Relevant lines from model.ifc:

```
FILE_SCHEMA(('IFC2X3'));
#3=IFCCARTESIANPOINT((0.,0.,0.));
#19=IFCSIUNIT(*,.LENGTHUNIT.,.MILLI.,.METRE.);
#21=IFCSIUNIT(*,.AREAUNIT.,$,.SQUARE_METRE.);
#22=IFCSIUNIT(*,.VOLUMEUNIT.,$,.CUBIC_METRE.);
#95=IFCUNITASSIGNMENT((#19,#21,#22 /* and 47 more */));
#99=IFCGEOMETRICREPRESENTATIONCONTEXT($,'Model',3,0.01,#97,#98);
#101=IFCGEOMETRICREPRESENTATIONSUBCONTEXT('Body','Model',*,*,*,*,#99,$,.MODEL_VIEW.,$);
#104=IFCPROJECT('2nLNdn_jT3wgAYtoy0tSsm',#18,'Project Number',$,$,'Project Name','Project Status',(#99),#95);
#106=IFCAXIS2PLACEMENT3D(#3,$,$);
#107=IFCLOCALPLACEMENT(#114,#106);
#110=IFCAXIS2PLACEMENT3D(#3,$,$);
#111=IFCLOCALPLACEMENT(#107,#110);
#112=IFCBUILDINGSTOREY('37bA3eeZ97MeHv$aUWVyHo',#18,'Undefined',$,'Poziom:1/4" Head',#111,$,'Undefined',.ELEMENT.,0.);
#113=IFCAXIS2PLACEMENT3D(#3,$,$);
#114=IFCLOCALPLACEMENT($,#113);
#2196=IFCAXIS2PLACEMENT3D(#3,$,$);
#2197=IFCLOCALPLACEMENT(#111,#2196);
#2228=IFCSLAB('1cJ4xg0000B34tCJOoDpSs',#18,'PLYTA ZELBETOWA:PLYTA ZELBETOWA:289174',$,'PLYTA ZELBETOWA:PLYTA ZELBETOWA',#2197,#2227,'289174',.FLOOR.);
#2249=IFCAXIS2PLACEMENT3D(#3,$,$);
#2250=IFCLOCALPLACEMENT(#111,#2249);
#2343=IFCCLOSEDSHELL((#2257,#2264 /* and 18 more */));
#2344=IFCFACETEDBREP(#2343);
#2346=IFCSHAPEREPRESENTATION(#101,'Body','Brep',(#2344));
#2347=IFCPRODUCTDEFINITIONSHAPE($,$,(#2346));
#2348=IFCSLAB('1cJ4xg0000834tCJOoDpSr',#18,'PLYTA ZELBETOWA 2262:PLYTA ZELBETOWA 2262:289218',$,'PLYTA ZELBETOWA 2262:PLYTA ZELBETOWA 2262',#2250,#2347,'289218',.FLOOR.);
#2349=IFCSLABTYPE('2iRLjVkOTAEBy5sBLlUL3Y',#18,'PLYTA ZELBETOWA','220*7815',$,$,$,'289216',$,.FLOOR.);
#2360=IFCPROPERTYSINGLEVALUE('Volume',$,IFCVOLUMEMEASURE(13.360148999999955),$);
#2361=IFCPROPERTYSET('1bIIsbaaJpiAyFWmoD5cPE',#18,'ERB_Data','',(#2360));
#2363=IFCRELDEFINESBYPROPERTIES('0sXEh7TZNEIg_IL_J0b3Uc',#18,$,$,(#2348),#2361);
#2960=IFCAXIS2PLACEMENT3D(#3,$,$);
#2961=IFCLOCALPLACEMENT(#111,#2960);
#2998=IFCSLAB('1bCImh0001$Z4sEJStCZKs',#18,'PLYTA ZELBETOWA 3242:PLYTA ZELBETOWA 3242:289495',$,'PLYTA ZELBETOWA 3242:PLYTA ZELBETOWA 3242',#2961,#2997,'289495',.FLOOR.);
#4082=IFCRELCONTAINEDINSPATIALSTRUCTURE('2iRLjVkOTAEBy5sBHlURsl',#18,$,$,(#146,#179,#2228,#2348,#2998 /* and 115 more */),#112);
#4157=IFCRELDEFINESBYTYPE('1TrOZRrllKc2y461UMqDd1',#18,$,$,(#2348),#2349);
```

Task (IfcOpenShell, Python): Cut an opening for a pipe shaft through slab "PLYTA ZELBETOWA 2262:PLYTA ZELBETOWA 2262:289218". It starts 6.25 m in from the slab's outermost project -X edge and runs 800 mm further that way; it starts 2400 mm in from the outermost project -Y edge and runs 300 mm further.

```python
import numpy as np
import ifcopenshell
import ifcopenshell.api.feature
import ifcopenshell.api.geometry
import ifcopenshell.api.pset
import ifcopenshell.api.root
import ifcopenshell.geom
import ifcopenshell.util.element
import ifcopenshell.util.placement
import ifcopenshell.util.representation
import ifcopenshell.util.shape
import ifcopenshell.util.unit

model = ifcopenshell.open("model.ifc")
unit_scale = ifcopenshell.util.unit.calculate_unit_scale(model)
volume_scale = ifcopenshell.util.unit.calculate_unit_scale(model, "VOLUMEUNIT")
settings = ifcopenshell.geom.settings()


def volume(element):
    """Net volume in cubic metres, openings subtracted."""
    shape = ifcopenshell.geom.create_shape(settings, element)
    return ifcopenshell.util.shape.get_volume(shape.geometry)


slab = model.by_id(2348)
before = volume(slab)

# Extent in the slab's own axes, in metres. The edges named are its -X and -Y sides.
slab_shape = ifcopenshell.geom.create_shape(settings, slab)
vertices = ifcopenshell.util.shape.get_vertices(slab_shape.geometry)
x_min, y_min, bottom = vertices.min(axis=0)
top = vertices[:, 2].max()

opening = ifcopenshell.api.root.create_entity(model, ifc_class="IfcOpeningElement", name="Pipe shaft opening")
context = ifcopenshell.util.representation.get_context(model, "Model", "Body", "MODEL_VIEW")
width, depth = 0.8, 0.3
outline = [(0.0, 0.0), (width, 0.0), (width, depth), (0.0, depth), (0.0, 0.0)]
# Overshoot both faces by 50 mm so the cut is clean.
shape = ifcopenshell.api.geometry.add_slab_representation(
    model, context=context, depth=top - bottom + 0.1, polyline=outline
)
ifcopenshell.api.geometry.assign_representation(model, product=opening, representation=shape)

matrix = ifcopenshell.util.placement.get_local_placement(slab.ObjectPlacement)
matrix[:, 3] = matrix @ np.append(np.array([x_min + 6.25, y_min + 2.4, bottom - 0.05]) / unit_scale, 1.0)
ifcopenshell.api.geometry.edit_object_placement(model, product=opening, matrix=matrix, is_si=False)
ifcopenshell.api.feature.add_feature(model, feature=opening, element=slab)

after = volume(slab)

# Update the slab's stored quantities.
pset = model.by_id(ifcopenshell.util.element.get_pset(slab, "ERB_Data", should_inherit=False)["id"])
ifcopenshell.api.pset.edit_pset(model, pset=pset, properties={
    "Volume": model.create_entity("IfcVolumeMeasure", after / volume_scale),
})

print(f"slab volume {before:.3f} -> {after:.3f} m3")

model.write("model_v2.ifc")
```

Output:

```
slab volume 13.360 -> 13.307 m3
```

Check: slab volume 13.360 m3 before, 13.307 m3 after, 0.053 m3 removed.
